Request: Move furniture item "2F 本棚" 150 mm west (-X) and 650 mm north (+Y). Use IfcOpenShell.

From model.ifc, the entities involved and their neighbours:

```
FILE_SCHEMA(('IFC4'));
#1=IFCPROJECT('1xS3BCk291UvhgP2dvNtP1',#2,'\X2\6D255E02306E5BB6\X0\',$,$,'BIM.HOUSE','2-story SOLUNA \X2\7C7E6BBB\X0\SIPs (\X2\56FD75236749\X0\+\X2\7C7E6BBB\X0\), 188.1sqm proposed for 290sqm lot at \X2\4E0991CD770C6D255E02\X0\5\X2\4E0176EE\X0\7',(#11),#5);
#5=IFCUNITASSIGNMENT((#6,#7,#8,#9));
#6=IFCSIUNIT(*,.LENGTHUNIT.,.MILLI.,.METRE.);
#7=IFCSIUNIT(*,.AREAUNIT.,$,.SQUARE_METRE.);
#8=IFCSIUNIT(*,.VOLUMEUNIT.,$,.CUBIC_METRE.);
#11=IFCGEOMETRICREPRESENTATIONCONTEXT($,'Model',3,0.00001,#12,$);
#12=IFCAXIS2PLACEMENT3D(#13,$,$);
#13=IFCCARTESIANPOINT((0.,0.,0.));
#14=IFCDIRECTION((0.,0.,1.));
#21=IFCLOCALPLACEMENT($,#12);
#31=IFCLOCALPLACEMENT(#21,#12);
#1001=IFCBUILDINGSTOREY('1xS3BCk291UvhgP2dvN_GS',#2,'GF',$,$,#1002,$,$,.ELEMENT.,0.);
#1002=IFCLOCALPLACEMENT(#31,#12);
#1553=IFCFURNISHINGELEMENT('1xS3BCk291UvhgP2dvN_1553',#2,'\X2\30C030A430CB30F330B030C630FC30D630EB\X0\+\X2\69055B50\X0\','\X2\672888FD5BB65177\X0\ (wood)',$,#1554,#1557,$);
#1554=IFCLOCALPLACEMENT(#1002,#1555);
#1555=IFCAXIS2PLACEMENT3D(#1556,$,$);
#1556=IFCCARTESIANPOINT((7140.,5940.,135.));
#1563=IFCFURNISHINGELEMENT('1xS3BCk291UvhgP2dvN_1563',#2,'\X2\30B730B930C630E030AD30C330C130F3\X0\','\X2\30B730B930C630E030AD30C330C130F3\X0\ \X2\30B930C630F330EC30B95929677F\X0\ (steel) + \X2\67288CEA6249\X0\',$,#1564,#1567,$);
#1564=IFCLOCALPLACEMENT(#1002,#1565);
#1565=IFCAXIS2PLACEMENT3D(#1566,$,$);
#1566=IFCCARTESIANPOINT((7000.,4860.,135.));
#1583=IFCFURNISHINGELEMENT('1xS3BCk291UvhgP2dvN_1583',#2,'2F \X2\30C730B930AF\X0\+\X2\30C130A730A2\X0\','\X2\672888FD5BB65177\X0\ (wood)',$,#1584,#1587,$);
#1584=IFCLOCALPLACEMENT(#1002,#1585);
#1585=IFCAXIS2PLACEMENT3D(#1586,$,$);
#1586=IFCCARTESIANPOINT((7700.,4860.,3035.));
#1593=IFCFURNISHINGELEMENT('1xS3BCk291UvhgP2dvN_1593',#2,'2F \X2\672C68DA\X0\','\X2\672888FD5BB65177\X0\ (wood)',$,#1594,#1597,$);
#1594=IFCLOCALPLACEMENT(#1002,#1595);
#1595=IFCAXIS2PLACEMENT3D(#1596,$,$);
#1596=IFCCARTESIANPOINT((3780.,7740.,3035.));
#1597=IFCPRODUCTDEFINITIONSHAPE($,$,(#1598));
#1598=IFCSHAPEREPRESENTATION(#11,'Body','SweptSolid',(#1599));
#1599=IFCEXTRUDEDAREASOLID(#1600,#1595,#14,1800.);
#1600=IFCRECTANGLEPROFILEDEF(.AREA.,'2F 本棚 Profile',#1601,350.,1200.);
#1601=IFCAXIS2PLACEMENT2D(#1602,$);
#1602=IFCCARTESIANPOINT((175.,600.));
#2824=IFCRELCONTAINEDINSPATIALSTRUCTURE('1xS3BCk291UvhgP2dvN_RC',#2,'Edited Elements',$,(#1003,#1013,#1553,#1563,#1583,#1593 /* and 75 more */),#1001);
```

```python
import ifcopenshell
import ifcopenshell.api.geometry
import ifcopenshell.util.placement

model = ifcopenshell.open("model.ifc")

item = model.by_guid("1xS3BCk291UvhgP2dvN_1593")
matrix = ifcopenshell.util.placement.get_local_placement(item.ObjectPlacement)
matrix[0, 3] -= 150.0
matrix[1, 3] += 650.0
ifcopenshell.api.geometry.edit_object_placement(model, product=item, matrix=matrix, is_si=False)

print(ifcopenshell.util.placement.get_local_placement(item.ObjectPlacement).round(3) + 0.0)

model.write("model_v2.ifc")
```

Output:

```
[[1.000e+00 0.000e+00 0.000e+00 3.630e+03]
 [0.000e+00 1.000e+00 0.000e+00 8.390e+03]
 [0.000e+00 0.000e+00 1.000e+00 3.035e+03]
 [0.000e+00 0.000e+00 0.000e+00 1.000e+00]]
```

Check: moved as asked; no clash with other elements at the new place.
